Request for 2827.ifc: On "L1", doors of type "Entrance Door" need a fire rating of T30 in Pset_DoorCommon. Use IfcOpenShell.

First a look at what the model holds.

```python
import ifcopenshell
import ifcopenshell.util.element

model = ifcopenshell.open("2827.ifc")
print(model.schema)
storey = next(s for s in model.by_type("IfcBuildingStorey") if s.Name == "L1")
doors = [e for e in ifcopenshell.util.element.get_decomposition(storey) if e.is_a("IfcDoor")]
seen = {}
for e in doors:
    element_type = ifcopenshell.util.element.get_type(e)
    key = (element_type.Name if element_type != e and element_type else None, ifcopenshell.util.element.get_pset(e, "Pset_DoorCommon", "FireRating"))
    seen[key] = seen.get(key, 0) + 1
for (name, value), count in sorted(seen.items(), key=str):
    print(count, "x", name, "|", value)
```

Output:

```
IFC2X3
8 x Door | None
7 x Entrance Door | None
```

```python
import ifcopenshell
import ifcopenshell.api.pset
import ifcopenshell.util.element

model = ifcopenshell.open("2827.ifc")

storey = next(s for s in model.by_type("IfcBuildingStorey") if s.Name == "L1")
doors = [e for e in ifcopenshell.util.element.get_decomposition(storey) if e.is_a("IfcDoor")]

count = 0
for e in doors:
    element_type = ifcopenshell.util.element.get_type(e)
    if element_type in (None, e) or element_type.Name != "Entrance Door":
        continue
    # add_pset returns the element's existing set when there is one.
    pset = ifcopenshell.api.pset.add_pset(model, product=e, name="Pset_DoorCommon")
    ifcopenshell.api.pset.edit_pset(model, pset=pset, properties={"FireRating": "T30"})
    count += 1

print(count, "doors updated")

model.write("2827-out.ifc")
```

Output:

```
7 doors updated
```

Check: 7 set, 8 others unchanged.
